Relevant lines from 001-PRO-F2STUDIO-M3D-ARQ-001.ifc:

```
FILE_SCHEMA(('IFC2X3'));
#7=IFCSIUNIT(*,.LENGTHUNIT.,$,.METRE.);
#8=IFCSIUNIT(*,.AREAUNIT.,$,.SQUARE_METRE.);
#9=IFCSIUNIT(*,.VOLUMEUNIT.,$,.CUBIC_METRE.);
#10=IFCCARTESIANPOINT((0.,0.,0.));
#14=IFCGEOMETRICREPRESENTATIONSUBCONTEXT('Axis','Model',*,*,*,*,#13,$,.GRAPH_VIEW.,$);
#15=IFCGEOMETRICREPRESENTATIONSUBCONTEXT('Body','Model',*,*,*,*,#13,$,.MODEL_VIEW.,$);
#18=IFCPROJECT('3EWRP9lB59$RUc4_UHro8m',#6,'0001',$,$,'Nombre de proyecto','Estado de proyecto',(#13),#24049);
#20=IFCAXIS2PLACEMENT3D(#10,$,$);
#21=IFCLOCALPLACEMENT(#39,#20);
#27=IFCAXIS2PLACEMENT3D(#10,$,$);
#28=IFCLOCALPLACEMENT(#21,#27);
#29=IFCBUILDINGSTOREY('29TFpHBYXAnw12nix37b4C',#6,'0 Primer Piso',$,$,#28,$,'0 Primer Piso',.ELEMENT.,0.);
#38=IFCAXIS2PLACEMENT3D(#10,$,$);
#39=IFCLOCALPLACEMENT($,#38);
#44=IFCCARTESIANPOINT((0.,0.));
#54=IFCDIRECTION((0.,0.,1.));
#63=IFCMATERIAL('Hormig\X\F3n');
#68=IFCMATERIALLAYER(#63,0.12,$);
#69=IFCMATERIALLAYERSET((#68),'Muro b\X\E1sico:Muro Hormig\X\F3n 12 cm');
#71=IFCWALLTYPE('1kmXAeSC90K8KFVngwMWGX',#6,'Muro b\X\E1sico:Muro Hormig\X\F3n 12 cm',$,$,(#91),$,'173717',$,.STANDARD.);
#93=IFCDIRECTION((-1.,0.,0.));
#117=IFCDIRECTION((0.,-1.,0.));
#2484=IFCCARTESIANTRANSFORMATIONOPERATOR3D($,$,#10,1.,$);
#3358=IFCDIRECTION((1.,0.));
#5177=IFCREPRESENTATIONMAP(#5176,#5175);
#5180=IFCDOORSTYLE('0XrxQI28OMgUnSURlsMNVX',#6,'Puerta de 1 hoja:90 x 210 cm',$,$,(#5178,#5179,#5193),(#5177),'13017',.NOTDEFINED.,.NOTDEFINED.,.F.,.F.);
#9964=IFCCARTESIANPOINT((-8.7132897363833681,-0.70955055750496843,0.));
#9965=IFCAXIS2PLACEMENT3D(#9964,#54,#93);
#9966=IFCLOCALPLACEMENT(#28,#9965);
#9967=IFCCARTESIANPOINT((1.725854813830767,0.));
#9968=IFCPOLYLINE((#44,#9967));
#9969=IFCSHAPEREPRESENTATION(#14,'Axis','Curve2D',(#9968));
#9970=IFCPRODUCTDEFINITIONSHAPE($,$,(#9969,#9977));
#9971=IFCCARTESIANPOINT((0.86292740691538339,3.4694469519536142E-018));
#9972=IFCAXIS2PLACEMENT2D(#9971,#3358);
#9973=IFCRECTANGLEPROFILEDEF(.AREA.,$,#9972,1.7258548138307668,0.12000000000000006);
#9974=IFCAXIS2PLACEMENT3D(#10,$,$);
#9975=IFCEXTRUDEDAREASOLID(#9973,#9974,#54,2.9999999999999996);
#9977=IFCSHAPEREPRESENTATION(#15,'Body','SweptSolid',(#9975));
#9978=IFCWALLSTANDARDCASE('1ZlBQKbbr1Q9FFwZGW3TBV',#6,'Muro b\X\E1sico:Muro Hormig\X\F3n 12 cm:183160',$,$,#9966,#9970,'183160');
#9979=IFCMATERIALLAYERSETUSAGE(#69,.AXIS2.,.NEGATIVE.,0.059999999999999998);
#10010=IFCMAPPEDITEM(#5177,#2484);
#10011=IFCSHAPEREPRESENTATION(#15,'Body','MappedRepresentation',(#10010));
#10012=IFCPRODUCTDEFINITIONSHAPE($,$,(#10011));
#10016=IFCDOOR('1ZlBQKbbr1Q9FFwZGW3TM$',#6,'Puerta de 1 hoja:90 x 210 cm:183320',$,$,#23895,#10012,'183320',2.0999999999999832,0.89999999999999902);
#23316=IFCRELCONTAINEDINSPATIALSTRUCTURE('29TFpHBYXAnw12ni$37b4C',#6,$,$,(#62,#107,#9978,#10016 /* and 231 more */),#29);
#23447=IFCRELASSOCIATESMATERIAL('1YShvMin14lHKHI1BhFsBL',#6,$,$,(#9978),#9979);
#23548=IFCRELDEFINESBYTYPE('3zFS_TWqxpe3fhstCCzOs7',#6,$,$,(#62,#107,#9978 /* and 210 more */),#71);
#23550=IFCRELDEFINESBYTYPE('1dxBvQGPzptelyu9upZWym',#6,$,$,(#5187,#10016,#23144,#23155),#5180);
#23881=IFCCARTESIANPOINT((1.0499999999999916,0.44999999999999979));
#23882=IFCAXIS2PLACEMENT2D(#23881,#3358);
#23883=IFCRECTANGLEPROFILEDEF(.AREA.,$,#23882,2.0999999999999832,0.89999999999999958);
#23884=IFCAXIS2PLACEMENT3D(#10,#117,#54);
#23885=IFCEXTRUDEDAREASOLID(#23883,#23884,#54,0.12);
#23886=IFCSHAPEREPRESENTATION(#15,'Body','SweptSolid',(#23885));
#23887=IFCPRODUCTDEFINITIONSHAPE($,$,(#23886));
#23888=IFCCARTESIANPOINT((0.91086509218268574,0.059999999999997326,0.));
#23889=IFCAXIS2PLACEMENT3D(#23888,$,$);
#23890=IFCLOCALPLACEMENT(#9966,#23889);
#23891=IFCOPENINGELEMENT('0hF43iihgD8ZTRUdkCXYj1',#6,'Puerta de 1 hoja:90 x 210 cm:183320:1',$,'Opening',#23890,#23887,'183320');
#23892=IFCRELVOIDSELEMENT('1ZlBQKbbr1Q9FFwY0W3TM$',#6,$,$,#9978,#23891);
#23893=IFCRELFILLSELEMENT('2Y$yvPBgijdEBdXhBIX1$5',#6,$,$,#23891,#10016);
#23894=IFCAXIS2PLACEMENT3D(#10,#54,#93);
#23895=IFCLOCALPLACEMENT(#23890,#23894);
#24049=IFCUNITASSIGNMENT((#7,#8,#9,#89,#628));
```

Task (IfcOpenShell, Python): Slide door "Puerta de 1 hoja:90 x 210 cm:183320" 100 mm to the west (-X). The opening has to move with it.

```python
import ifcopenshell
import ifcopenshell.api.geometry
import ifcopenshell.util.placement
import ifcopenshell.util.unit

model = ifcopenshell.open("001-PRO-F2STUDIO-M3D-ARQ-001.ifc")
unit_scale = ifcopenshell.util.unit.calculate_unit_scale(model)

door = model.by_id(10016)
opening = door.FillsVoids[0].RelatingOpeningElement
wall = opening.VoidsElements[0].RelatingBuildingElement

wall_matrix = ifcopenshell.util.placement.get_local_placement(wall.ObjectPlacement)
shift = wall_matrix[:3, 0] * 0.1 / unit_scale
before = ifcopenshell.util.placement.get_local_placement(door.ObjectPlacement)[:3, 3].copy()

# The door is placed relative to its opening, so it follows when the opening moves.
matrix = ifcopenshell.util.placement.get_local_placement(opening.ObjectPlacement)
matrix[:3, 3] += shift
ifcopenshell.api.geometry.edit_object_placement(
    model, product=opening, matrix=matrix, is_si=False, should_transform_children=True
)

after = ifcopenshell.util.placement.get_local_placement(door.ObjectPlacement)[:3, 3]
print("door moved by", (after - before).round(3) + 0.0)

model.write("001-PRO-F2STUDIO-M3D-ARQ-001_v2.ifc")
```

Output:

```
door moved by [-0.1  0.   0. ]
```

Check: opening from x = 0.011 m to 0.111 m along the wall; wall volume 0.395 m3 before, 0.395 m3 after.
